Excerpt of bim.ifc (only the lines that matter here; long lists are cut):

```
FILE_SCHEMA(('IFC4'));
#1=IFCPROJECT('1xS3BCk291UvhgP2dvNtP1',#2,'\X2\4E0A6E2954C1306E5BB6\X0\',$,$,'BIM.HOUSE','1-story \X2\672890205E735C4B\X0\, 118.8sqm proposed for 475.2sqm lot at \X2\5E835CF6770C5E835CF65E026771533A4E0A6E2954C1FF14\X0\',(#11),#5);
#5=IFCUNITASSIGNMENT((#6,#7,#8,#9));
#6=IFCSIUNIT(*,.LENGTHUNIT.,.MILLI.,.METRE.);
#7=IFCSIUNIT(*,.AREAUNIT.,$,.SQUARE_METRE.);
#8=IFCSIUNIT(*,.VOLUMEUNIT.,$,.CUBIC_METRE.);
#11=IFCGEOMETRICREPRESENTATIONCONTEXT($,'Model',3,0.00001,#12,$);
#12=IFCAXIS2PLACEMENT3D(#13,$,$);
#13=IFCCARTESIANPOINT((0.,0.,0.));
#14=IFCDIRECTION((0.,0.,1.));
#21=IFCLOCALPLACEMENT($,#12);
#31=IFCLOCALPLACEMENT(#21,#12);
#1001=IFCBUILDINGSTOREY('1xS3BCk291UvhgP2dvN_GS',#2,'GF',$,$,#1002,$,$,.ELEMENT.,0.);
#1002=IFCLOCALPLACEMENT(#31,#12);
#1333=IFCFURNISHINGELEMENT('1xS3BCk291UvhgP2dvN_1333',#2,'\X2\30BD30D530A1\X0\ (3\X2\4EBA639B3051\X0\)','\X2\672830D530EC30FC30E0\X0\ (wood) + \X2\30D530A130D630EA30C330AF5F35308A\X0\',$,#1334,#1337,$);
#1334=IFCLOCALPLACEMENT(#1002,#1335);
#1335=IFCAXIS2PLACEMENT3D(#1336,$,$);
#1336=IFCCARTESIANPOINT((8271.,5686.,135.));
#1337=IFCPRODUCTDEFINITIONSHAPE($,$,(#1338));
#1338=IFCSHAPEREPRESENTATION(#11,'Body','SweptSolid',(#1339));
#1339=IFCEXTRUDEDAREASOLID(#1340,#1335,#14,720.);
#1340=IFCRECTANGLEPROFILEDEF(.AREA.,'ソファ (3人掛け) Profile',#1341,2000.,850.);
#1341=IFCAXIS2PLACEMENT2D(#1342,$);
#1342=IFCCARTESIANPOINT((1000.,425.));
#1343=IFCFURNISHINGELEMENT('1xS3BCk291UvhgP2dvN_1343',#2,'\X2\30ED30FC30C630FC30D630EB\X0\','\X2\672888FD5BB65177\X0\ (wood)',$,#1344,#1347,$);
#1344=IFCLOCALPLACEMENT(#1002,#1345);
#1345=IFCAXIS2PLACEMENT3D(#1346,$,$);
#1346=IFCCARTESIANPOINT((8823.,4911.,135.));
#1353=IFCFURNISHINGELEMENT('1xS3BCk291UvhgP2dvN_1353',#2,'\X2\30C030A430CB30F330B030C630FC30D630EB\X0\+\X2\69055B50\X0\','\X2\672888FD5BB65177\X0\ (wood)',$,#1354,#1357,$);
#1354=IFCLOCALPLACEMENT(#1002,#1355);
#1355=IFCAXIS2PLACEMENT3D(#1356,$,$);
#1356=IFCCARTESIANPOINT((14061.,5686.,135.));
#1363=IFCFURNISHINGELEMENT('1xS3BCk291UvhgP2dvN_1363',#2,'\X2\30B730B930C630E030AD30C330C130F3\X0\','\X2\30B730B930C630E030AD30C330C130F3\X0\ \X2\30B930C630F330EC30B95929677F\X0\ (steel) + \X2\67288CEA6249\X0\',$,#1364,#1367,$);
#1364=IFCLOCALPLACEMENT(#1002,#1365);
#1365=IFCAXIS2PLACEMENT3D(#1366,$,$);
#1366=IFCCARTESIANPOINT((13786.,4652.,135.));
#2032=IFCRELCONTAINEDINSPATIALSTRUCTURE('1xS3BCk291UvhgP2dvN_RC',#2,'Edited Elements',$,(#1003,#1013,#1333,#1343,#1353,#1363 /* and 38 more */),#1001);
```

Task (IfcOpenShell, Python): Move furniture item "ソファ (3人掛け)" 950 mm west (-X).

```python
import ifcopenshell
import ifcopenshell.api.geometry
import ifcopenshell.util.placement
import ifcopenshell.util.unit

model = ifcopenshell.open("bim.ifc")
unit_scale = ifcopenshell.util.unit.calculate_unit_scale(model)

item = model.by_id(1333)
matrix = ifcopenshell.util.placement.get_local_placement(item.ObjectPlacement)
matrix[0, 3] -= 0.95 / unit_scale
ifcopenshell.api.geometry.edit_object_placement(model, product=item, matrix=matrix, is_si=False)

print(ifcopenshell.util.placement.get_local_placement(item.ObjectPlacement).round(3) + 0.0)

model.write("bim_edited.ifc")
```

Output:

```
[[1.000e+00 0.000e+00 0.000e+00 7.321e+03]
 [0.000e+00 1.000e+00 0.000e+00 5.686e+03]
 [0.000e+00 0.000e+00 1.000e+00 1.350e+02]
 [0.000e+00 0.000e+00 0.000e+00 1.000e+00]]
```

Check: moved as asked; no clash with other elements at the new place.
